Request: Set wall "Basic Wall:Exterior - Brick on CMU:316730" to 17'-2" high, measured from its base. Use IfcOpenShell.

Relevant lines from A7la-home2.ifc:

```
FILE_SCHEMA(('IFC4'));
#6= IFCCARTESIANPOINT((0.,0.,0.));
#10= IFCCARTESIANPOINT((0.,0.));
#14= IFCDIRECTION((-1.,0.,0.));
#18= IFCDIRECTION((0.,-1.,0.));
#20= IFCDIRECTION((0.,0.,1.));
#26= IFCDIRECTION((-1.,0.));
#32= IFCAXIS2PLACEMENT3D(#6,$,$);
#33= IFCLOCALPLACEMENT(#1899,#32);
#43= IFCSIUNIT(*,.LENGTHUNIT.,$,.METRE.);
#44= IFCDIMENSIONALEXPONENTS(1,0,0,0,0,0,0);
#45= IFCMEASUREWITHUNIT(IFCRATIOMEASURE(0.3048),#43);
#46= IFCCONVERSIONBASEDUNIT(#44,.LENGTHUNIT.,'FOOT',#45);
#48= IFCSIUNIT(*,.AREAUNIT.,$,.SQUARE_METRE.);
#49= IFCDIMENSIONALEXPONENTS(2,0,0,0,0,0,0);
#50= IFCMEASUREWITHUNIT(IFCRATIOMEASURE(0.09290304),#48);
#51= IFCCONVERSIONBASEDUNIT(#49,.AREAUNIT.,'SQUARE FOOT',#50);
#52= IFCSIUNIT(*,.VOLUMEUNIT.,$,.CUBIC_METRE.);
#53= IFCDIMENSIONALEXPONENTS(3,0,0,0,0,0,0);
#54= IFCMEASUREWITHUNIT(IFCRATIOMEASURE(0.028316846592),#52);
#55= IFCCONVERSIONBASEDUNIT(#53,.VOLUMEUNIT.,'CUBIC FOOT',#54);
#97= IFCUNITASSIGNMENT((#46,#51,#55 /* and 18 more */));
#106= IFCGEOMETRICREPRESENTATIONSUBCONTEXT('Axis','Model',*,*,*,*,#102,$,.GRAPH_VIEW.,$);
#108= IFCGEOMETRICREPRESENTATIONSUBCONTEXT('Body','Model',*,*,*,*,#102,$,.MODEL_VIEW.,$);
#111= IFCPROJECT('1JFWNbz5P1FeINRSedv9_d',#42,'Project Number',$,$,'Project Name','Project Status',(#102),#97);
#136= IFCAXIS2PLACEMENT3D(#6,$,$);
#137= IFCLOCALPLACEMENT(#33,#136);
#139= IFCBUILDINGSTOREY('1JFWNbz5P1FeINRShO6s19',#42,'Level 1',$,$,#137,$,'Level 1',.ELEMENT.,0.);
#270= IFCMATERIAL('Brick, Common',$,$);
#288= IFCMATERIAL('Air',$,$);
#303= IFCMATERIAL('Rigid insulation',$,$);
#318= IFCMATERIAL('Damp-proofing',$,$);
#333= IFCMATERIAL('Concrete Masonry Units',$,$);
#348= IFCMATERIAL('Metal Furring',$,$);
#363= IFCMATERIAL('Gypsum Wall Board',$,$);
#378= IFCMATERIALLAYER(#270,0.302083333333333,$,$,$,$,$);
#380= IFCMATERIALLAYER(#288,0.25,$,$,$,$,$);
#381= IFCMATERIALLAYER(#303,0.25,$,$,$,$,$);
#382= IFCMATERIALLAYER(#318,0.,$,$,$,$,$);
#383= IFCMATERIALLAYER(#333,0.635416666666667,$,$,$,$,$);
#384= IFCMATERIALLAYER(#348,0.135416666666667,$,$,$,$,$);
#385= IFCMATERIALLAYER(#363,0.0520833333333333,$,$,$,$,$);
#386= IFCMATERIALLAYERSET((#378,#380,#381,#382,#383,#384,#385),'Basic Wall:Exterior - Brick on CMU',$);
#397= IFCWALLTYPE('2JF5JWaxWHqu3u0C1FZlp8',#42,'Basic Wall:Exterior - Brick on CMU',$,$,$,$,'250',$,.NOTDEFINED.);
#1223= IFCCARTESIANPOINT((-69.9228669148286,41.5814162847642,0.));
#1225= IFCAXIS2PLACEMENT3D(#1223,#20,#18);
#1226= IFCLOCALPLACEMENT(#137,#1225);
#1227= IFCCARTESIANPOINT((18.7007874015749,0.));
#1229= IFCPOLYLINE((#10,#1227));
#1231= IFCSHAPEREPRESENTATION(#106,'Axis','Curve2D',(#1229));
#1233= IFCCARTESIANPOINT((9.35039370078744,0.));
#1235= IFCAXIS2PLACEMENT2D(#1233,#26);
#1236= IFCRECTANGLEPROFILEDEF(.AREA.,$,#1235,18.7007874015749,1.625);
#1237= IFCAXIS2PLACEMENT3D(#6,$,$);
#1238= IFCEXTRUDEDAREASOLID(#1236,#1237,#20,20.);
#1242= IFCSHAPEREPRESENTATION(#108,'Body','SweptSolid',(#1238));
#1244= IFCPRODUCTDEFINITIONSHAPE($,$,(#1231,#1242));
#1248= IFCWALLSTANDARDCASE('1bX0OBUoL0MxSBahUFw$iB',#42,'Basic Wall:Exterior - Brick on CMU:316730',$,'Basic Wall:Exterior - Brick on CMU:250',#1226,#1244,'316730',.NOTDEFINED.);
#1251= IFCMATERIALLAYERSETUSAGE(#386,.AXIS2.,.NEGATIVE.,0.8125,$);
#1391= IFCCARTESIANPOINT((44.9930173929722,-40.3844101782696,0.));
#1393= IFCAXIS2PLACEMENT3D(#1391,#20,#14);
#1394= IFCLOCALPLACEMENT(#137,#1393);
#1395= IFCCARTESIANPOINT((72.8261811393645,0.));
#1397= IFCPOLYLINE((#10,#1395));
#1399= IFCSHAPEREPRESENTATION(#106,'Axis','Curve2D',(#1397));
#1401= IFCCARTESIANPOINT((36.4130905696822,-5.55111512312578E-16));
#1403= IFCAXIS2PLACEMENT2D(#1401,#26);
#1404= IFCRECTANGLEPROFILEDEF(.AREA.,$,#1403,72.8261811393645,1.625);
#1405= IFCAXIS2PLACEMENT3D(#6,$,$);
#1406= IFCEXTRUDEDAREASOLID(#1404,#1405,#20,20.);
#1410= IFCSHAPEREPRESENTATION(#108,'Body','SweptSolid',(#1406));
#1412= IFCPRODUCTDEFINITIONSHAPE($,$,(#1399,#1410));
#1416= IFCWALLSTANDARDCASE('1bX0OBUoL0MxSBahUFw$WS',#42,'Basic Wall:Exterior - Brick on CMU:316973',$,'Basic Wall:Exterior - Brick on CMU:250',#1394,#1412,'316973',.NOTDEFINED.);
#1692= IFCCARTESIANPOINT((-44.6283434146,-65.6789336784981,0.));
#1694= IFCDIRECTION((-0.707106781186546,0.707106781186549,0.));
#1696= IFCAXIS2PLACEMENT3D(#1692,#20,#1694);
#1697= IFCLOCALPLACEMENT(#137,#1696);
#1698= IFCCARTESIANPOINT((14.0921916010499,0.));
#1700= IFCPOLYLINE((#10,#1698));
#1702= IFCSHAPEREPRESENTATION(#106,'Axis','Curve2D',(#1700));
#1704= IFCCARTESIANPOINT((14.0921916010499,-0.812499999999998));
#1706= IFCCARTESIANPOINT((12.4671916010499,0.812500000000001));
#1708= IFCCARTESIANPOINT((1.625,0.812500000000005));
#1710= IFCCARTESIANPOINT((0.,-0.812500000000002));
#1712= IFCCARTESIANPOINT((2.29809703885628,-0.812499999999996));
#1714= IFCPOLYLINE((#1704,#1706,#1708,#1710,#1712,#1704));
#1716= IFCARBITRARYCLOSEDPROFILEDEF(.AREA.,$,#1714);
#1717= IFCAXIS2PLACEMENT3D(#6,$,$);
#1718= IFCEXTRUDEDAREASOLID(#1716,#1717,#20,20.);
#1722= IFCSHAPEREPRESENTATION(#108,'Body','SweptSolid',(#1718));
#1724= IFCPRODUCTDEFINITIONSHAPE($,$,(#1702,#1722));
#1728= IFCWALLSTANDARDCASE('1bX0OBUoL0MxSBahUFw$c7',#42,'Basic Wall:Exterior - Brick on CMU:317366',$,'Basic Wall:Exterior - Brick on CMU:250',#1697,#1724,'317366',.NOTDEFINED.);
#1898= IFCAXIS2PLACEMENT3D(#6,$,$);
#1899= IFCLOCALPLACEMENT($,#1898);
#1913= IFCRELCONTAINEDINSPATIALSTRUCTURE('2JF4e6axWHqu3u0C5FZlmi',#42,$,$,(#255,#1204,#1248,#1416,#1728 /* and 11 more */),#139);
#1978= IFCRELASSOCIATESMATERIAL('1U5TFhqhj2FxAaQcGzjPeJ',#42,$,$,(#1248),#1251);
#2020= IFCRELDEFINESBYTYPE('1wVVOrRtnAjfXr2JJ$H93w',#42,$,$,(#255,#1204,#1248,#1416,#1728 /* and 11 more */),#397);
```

```python
import ifcopenshell
import ifcopenshell.geom
import ifcopenshell.util.representation
import ifcopenshell.util.shape
import ifcopenshell.util.unit

model = ifcopenshell.open("A7la-home2.ifc")
unit_scale = ifcopenshell.util.unit.calculate_unit_scale(model)
settings = ifcopenshell.geom.settings()


def volume(element):
    """Net volume in cubic metres, openings subtracted."""
    shape = ifcopenshell.geom.create_shape(settings, element)
    return ifcopenshell.util.shape.get_volume(shape.geometry)


wall = model.by_guid("1bX0OBUoL0MxSBahUFw$iB")
before = volume(wall)

body = ifcopenshell.util.representation.get_representation(wall, "Model", "Body")
solid = body.Items[0]
old_height = solid.Depth
solid.Depth = 206 * 0.0254 / unit_scale
after = volume(wall)

print(f"height {old_height:g} -> {solid.Depth:g}, volume {before:.3f} -> {after:.3f} m3")

model.write("A7la-home2_edited.ifc")
```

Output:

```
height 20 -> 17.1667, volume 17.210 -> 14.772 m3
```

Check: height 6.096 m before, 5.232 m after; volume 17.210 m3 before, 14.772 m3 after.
